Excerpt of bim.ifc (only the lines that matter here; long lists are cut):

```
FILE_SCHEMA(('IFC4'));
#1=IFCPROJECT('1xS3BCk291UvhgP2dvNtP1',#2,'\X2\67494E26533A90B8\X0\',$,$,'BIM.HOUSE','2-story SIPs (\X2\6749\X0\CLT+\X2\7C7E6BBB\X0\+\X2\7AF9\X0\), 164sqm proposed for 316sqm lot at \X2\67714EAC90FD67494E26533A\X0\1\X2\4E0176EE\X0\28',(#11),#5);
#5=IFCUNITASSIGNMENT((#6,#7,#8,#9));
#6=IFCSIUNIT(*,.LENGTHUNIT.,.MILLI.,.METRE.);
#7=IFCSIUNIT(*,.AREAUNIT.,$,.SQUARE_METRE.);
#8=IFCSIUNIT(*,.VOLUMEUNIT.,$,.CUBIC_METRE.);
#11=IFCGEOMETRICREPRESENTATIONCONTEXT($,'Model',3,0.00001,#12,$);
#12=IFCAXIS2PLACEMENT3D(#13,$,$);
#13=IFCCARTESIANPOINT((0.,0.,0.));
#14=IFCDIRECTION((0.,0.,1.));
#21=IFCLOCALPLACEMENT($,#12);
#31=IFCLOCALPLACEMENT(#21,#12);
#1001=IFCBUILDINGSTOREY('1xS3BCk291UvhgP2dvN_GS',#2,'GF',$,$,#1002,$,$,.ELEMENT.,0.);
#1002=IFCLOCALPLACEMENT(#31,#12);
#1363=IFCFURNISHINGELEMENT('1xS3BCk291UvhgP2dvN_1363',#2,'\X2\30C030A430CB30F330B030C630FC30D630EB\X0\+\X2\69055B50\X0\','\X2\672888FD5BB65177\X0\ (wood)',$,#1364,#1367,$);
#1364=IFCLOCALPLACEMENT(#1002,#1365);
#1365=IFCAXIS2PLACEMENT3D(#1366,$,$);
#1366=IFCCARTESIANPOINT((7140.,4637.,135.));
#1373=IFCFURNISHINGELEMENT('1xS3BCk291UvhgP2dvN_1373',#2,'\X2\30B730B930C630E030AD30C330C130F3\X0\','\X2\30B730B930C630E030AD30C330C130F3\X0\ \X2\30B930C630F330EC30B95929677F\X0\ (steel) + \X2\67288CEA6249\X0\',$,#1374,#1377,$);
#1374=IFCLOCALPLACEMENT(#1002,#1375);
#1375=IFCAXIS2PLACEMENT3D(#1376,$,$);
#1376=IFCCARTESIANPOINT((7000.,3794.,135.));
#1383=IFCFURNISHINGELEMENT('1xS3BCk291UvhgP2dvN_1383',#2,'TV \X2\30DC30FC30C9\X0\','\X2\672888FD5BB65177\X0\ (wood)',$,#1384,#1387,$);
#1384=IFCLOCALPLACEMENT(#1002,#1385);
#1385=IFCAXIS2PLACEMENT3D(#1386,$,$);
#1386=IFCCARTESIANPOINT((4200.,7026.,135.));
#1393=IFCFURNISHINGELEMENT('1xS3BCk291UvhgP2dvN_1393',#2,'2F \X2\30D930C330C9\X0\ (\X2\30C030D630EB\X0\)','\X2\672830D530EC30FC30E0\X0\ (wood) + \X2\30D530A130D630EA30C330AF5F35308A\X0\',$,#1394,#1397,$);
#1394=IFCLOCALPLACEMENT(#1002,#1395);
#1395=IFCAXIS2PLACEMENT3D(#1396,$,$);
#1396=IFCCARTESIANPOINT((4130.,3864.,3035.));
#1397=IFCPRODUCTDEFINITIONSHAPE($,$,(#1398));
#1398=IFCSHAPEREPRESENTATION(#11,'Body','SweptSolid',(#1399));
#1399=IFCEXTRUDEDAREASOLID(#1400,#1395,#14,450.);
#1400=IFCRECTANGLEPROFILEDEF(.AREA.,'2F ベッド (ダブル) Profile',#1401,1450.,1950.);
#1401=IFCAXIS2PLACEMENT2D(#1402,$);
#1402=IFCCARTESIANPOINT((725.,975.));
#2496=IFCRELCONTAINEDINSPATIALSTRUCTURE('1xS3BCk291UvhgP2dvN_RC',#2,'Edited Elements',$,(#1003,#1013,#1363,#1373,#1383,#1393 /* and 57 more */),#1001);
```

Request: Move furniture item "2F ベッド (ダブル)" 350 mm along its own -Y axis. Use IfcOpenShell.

```python
import ifcopenshell
import ifcopenshell.api.geometry
import ifcopenshell.util.placement
import ifcopenshell.util.unit

model = ifcopenshell.open("bim.ifc")
unit_scale = ifcopenshell.util.unit.calculate_unit_scale(model)

item = model.by_guid("1xS3BCk291UvhgP2dvN_1393")
matrix = ifcopenshell.util.placement.get_local_placement(item.ObjectPlacement)
matrix[:3, 3] -= matrix[:3, 1] * 0.35 / unit_scale
ifcopenshell.api.geometry.edit_object_placement(model, product=item, matrix=matrix, is_si=False)

print(ifcopenshell.util.placement.get_local_placement(item.ObjectPlacement).round(3) + 0.0)

model.write("bim-out.ifc")
```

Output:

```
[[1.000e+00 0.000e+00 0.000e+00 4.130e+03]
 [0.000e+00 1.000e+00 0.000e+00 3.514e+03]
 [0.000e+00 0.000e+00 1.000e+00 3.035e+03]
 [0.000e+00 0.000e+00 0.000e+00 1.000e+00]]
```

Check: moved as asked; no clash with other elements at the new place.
